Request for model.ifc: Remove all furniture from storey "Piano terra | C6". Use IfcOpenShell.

First a look at what the model holds.

```python
import ifcopenshell
import ifcopenshell.util.element

model = ifcopenshell.open("model.ifc")
print(model.schema)
storey = next(s for s in model.by_type("IfcBuildingStorey") if s.Name == "Piano terra | C6")
furniture = [e for e in ifcopenshell.util.element.get_decomposition(storey) if e.is_a("IfcFurnishingElement")]
seen = {}
for e in furniture:
    element_type = ifcopenshell.util.element.get_type(e)
    name = element_type.Name if element_type not in (None, e) else None
    seen[name] = seen.get(name, 0) + 1
for name, count in sorted(seen.items(), key=str):
    print(count, "x", name)
```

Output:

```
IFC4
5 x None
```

```python
import ifcopenshell
import ifcopenshell.api.root
import ifcopenshell.util.element

model = ifcopenshell.open("model.ifc")

storey = next(s for s in model.by_type("IfcBuildingStorey") if s.Name == "Piano terra | C6")
furniture = [e for e in ifcopenshell.util.element.get_decomposition(storey) if e.is_a("IfcFurnishingElement")]

for e in furniture:
    ifcopenshell.api.root.remove_product(model, product=e)
print(len(furniture), "removed")

model.write("model-out.ifc")
```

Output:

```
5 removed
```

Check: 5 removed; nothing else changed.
